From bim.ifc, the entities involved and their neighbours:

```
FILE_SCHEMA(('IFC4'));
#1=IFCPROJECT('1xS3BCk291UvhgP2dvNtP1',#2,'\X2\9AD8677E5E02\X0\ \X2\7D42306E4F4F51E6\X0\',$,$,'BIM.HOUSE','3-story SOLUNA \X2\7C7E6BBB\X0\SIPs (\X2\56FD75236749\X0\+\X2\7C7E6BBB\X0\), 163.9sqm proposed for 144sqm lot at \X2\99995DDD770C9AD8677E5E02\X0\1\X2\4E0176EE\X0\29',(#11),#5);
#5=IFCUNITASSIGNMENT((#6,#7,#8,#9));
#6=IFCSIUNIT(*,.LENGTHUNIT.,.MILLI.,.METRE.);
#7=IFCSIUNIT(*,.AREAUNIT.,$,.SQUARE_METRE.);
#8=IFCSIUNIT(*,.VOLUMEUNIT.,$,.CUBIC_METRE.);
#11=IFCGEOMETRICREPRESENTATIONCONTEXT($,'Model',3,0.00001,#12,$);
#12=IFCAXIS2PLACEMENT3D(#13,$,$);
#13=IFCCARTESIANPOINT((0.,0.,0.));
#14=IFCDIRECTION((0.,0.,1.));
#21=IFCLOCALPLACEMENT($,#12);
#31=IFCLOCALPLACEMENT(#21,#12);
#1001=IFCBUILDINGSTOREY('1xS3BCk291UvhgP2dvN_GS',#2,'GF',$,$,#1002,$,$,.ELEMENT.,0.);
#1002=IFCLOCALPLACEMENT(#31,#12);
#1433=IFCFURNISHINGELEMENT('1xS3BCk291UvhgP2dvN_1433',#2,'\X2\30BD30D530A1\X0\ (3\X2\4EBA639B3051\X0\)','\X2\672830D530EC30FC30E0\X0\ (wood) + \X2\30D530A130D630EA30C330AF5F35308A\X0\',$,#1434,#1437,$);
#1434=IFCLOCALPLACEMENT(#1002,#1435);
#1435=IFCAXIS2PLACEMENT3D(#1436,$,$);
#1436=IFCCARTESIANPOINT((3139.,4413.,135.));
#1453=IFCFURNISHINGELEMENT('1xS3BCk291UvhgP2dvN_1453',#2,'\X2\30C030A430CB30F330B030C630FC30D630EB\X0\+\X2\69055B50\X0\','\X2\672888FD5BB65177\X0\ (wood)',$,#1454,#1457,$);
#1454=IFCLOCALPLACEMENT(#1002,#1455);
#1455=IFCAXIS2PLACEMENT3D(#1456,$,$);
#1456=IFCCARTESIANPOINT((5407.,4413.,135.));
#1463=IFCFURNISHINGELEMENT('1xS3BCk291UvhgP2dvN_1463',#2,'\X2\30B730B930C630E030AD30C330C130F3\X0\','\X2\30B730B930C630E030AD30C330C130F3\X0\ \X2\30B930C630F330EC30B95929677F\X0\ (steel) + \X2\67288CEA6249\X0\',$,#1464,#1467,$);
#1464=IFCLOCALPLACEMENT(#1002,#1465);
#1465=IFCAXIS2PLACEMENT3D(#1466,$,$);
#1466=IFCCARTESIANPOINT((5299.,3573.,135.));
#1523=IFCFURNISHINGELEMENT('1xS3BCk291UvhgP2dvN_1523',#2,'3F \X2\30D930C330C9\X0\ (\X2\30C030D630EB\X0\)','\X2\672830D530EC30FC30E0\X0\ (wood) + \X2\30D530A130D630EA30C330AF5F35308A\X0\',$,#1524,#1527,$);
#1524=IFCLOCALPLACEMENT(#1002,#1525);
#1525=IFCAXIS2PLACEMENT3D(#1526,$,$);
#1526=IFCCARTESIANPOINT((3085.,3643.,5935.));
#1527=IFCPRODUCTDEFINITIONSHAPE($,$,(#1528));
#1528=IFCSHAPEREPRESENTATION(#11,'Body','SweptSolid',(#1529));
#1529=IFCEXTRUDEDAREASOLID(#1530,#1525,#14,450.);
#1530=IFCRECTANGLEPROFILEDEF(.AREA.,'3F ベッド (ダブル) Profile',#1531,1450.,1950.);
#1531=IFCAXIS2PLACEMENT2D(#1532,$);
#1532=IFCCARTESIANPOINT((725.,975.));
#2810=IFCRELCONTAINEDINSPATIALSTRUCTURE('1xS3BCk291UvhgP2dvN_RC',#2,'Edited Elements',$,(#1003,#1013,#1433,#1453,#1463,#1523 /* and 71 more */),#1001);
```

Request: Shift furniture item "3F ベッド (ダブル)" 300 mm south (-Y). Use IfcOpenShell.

```python
import ifcopenshell
import ifcopenshell.api.geometry
import ifcopenshell.util.placement

model = ifcopenshell.open("bim.ifc")

item = model.by_guid("1xS3BCk291UvhgP2dvN_1523")
matrix = ifcopenshell.util.placement.get_local_placement(item.ObjectPlacement)
matrix[1, 3] -= 300.0
ifcopenshell.api.geometry.edit_object_placement(model, product=item, matrix=matrix, is_si=False)

print(ifcopenshell.util.placement.get_local_placement(item.ObjectPlacement).round(3) + 0.0)

model.write("bim_v2.ifc")
```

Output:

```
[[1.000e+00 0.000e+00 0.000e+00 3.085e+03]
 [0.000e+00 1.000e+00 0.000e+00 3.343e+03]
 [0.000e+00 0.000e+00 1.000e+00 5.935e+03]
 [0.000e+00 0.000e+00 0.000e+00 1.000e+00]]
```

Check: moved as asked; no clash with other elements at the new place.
